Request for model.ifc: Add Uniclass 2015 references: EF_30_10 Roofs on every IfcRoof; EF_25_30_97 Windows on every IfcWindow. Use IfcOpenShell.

First a look at what the model holds.

```python
import ifcopenshell

model = ifcopenshell.open("model.ifc")
print(model.schema)
print("classifications:", [c.Name for c in model.by_type("IfcClassification")])
for ifc_class in ("IfcDoor", "IfcRoof", "IfcStair", "IfcWall", "IfcWindow"):
    print(ifc_class, len(model.by_type(ifc_class)))
```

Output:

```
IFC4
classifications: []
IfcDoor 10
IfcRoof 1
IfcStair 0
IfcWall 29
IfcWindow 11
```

```python
import ifcopenshell
import ifcopenshell.api.classification

model = ifcopenshell.open("model.ifc")

system = ifcopenshell.api.classification.add_classification(model, classification="Uniclass 2015")

codes = {
    "IfcRoof": ("EF_30_10", "Roofs"),
    "IfcWindow": ("EF_25_30_97", "Windows"),
}
for ifc_class, (code, name) in codes.items():
    products = model.by_type(ifc_class)
    ifcopenshell.api.classification.add_reference(
        model, products=products, classification=system, identification=code, name=name
    )
    print(code, len(products))

model.write("model-out.ifc")
```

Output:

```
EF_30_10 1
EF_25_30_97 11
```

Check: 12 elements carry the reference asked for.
